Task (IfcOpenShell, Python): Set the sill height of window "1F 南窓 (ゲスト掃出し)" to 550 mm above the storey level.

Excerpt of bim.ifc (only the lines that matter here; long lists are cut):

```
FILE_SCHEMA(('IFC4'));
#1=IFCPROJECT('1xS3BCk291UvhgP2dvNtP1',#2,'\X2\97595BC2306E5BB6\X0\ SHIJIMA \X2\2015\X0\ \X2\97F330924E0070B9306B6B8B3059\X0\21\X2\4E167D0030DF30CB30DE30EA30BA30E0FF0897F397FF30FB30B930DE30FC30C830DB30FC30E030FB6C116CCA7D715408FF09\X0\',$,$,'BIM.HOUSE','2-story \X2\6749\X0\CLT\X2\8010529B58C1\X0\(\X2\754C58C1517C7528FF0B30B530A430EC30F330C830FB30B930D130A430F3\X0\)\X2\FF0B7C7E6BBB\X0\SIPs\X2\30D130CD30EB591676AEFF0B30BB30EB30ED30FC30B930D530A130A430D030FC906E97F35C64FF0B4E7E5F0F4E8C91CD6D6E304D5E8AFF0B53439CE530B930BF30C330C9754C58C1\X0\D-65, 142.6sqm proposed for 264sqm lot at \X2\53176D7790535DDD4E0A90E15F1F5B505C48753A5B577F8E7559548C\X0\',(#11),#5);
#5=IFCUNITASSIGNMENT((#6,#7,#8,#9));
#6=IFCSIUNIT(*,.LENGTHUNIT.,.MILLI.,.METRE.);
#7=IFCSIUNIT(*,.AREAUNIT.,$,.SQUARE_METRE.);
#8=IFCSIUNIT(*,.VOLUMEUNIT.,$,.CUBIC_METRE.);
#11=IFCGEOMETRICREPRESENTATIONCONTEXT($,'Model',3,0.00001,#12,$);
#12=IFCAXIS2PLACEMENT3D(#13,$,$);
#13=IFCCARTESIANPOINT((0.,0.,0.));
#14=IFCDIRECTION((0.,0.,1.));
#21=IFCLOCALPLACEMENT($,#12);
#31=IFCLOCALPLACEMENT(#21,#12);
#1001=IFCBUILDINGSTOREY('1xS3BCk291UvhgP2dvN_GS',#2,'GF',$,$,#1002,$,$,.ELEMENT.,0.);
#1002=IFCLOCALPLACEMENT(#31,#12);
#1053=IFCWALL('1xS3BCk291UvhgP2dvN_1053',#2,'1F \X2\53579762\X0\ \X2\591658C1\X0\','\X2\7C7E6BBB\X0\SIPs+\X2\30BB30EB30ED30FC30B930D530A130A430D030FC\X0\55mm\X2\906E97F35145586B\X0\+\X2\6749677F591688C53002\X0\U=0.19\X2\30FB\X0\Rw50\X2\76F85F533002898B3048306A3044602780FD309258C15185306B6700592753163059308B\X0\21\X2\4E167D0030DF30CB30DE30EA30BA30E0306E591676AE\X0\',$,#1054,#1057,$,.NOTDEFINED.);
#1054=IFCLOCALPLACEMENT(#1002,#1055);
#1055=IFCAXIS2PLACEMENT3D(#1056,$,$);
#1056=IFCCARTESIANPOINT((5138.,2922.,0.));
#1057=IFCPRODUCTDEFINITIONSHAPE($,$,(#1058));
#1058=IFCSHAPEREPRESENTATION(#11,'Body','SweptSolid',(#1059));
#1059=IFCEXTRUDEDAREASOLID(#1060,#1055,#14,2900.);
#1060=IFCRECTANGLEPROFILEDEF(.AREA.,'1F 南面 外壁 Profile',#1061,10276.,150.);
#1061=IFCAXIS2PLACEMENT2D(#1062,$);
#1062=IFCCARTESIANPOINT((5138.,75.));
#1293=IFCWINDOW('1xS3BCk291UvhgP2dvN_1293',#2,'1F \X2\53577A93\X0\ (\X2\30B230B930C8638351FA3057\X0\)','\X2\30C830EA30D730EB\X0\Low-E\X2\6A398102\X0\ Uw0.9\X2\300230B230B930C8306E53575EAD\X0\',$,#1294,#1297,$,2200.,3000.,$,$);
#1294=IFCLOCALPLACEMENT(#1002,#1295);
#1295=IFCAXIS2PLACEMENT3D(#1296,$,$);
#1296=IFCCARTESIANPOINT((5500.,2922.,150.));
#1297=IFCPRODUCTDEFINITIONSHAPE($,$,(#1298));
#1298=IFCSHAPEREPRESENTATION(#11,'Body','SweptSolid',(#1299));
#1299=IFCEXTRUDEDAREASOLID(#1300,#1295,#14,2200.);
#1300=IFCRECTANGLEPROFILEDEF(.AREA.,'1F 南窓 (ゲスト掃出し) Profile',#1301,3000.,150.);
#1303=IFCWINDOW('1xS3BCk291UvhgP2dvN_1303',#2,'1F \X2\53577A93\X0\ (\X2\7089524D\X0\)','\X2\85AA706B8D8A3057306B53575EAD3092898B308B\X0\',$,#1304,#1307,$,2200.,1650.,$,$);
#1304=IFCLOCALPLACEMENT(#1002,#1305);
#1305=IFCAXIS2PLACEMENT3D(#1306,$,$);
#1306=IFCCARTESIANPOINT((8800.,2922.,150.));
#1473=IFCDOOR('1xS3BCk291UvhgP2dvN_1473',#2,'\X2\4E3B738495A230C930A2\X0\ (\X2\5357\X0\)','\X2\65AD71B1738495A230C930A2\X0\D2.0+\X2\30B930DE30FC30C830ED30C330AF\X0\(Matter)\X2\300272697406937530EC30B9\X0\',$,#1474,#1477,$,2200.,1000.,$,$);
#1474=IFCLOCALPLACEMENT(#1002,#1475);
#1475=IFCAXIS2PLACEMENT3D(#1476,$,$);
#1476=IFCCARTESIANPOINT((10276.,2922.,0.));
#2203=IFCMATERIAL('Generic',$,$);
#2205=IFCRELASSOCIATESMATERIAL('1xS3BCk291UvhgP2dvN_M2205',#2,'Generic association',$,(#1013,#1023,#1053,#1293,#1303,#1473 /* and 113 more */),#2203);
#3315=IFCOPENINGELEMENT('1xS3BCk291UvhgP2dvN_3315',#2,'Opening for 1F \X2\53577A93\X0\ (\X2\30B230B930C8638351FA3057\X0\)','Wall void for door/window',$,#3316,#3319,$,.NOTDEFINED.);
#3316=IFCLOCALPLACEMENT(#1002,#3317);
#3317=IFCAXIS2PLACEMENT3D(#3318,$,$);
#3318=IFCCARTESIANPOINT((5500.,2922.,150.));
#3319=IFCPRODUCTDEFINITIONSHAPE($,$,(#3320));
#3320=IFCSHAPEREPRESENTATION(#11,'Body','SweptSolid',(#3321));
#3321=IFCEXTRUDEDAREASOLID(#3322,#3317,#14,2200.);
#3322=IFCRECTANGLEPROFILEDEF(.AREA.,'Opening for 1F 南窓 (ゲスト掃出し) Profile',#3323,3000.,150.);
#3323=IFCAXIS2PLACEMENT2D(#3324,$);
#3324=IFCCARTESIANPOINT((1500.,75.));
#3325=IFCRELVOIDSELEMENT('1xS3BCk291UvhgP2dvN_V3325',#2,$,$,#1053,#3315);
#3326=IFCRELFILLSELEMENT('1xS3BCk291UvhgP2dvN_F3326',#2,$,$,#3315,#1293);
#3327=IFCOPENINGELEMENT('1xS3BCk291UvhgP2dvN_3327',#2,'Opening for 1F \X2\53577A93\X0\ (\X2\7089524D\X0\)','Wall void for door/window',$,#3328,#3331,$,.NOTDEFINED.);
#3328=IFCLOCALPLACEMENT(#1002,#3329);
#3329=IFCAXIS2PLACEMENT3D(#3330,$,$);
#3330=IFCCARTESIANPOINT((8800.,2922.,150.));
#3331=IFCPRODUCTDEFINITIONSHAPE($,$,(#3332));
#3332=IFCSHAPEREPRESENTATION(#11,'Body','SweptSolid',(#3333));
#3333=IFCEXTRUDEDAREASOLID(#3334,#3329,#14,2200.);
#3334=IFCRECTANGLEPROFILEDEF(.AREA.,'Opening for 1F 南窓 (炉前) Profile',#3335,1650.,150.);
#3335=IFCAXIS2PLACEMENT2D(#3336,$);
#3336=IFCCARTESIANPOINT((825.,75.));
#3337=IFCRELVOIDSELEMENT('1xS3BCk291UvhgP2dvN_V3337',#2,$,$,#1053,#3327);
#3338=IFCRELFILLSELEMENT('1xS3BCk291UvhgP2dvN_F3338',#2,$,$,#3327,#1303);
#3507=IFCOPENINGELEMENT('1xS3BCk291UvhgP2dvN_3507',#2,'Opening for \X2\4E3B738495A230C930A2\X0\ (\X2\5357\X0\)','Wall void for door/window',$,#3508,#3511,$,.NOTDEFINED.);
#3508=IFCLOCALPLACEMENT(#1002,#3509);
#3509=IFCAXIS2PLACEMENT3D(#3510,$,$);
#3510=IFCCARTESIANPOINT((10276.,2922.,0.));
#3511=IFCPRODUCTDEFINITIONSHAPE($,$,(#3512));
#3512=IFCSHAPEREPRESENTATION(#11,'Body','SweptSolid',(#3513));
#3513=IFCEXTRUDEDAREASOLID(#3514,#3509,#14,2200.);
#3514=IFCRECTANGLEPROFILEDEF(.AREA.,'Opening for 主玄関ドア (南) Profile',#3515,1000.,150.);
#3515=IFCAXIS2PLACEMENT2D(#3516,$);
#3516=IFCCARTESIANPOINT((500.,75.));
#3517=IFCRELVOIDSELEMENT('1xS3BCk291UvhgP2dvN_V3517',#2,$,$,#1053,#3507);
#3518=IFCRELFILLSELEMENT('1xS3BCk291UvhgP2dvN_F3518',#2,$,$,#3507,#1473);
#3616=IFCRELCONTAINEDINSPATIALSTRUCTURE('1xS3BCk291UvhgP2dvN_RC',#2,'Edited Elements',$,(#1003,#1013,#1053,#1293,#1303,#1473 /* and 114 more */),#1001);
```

```python
import numpy as np
import ifcopenshell
import ifcopenshell.api.geometry
import ifcopenshell.geom
import ifcopenshell.util.element
import ifcopenshell.util.placement
import ifcopenshell.util.shape
import ifcopenshell.util.unit

model = ifcopenshell.open("bim.ifc")
unit_scale = ifcopenshell.util.unit.calculate_unit_scale(model)

window = model.by_guid("1xS3BCk291UvhgP2dvN_1293")
opening = window.FillsVoids[0].RelatingOpeningElement
storey = ifcopenshell.util.element.get_container(window, ifc_class="IfcBuildingStorey")
level = ifcopenshell.util.placement.get_local_placement(storey.ObjectPlacement)[2, 3]

# The opening's origin need not be at the sill, so measure its lowest point.
shape = ifcopenshell.geom.create_shape(ifcopenshell.geom.settings(), opening)
bottom = ifcopenshell.util.shape.get_shape_bottom_elevation(shape, shape.geometry) / unit_scale
dz = level + 550.0 - bottom

shift = np.array([0.0, 0.0, dz])
# The window is not placed relative to its opening, so move both.
for product in (opening, window):
    matrix = ifcopenshell.util.placement.get_local_placement(product.ObjectPlacement)
    matrix[:3, 3] += shift
    ifcopenshell.api.geometry.edit_object_placement(model, product=product, matrix=matrix, is_si=False)

print(f"moved by {dz * unit_scale:+.3f} m")

model.write("bim_updated.ifc")
```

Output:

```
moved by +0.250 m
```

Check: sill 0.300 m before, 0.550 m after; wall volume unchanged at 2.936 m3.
